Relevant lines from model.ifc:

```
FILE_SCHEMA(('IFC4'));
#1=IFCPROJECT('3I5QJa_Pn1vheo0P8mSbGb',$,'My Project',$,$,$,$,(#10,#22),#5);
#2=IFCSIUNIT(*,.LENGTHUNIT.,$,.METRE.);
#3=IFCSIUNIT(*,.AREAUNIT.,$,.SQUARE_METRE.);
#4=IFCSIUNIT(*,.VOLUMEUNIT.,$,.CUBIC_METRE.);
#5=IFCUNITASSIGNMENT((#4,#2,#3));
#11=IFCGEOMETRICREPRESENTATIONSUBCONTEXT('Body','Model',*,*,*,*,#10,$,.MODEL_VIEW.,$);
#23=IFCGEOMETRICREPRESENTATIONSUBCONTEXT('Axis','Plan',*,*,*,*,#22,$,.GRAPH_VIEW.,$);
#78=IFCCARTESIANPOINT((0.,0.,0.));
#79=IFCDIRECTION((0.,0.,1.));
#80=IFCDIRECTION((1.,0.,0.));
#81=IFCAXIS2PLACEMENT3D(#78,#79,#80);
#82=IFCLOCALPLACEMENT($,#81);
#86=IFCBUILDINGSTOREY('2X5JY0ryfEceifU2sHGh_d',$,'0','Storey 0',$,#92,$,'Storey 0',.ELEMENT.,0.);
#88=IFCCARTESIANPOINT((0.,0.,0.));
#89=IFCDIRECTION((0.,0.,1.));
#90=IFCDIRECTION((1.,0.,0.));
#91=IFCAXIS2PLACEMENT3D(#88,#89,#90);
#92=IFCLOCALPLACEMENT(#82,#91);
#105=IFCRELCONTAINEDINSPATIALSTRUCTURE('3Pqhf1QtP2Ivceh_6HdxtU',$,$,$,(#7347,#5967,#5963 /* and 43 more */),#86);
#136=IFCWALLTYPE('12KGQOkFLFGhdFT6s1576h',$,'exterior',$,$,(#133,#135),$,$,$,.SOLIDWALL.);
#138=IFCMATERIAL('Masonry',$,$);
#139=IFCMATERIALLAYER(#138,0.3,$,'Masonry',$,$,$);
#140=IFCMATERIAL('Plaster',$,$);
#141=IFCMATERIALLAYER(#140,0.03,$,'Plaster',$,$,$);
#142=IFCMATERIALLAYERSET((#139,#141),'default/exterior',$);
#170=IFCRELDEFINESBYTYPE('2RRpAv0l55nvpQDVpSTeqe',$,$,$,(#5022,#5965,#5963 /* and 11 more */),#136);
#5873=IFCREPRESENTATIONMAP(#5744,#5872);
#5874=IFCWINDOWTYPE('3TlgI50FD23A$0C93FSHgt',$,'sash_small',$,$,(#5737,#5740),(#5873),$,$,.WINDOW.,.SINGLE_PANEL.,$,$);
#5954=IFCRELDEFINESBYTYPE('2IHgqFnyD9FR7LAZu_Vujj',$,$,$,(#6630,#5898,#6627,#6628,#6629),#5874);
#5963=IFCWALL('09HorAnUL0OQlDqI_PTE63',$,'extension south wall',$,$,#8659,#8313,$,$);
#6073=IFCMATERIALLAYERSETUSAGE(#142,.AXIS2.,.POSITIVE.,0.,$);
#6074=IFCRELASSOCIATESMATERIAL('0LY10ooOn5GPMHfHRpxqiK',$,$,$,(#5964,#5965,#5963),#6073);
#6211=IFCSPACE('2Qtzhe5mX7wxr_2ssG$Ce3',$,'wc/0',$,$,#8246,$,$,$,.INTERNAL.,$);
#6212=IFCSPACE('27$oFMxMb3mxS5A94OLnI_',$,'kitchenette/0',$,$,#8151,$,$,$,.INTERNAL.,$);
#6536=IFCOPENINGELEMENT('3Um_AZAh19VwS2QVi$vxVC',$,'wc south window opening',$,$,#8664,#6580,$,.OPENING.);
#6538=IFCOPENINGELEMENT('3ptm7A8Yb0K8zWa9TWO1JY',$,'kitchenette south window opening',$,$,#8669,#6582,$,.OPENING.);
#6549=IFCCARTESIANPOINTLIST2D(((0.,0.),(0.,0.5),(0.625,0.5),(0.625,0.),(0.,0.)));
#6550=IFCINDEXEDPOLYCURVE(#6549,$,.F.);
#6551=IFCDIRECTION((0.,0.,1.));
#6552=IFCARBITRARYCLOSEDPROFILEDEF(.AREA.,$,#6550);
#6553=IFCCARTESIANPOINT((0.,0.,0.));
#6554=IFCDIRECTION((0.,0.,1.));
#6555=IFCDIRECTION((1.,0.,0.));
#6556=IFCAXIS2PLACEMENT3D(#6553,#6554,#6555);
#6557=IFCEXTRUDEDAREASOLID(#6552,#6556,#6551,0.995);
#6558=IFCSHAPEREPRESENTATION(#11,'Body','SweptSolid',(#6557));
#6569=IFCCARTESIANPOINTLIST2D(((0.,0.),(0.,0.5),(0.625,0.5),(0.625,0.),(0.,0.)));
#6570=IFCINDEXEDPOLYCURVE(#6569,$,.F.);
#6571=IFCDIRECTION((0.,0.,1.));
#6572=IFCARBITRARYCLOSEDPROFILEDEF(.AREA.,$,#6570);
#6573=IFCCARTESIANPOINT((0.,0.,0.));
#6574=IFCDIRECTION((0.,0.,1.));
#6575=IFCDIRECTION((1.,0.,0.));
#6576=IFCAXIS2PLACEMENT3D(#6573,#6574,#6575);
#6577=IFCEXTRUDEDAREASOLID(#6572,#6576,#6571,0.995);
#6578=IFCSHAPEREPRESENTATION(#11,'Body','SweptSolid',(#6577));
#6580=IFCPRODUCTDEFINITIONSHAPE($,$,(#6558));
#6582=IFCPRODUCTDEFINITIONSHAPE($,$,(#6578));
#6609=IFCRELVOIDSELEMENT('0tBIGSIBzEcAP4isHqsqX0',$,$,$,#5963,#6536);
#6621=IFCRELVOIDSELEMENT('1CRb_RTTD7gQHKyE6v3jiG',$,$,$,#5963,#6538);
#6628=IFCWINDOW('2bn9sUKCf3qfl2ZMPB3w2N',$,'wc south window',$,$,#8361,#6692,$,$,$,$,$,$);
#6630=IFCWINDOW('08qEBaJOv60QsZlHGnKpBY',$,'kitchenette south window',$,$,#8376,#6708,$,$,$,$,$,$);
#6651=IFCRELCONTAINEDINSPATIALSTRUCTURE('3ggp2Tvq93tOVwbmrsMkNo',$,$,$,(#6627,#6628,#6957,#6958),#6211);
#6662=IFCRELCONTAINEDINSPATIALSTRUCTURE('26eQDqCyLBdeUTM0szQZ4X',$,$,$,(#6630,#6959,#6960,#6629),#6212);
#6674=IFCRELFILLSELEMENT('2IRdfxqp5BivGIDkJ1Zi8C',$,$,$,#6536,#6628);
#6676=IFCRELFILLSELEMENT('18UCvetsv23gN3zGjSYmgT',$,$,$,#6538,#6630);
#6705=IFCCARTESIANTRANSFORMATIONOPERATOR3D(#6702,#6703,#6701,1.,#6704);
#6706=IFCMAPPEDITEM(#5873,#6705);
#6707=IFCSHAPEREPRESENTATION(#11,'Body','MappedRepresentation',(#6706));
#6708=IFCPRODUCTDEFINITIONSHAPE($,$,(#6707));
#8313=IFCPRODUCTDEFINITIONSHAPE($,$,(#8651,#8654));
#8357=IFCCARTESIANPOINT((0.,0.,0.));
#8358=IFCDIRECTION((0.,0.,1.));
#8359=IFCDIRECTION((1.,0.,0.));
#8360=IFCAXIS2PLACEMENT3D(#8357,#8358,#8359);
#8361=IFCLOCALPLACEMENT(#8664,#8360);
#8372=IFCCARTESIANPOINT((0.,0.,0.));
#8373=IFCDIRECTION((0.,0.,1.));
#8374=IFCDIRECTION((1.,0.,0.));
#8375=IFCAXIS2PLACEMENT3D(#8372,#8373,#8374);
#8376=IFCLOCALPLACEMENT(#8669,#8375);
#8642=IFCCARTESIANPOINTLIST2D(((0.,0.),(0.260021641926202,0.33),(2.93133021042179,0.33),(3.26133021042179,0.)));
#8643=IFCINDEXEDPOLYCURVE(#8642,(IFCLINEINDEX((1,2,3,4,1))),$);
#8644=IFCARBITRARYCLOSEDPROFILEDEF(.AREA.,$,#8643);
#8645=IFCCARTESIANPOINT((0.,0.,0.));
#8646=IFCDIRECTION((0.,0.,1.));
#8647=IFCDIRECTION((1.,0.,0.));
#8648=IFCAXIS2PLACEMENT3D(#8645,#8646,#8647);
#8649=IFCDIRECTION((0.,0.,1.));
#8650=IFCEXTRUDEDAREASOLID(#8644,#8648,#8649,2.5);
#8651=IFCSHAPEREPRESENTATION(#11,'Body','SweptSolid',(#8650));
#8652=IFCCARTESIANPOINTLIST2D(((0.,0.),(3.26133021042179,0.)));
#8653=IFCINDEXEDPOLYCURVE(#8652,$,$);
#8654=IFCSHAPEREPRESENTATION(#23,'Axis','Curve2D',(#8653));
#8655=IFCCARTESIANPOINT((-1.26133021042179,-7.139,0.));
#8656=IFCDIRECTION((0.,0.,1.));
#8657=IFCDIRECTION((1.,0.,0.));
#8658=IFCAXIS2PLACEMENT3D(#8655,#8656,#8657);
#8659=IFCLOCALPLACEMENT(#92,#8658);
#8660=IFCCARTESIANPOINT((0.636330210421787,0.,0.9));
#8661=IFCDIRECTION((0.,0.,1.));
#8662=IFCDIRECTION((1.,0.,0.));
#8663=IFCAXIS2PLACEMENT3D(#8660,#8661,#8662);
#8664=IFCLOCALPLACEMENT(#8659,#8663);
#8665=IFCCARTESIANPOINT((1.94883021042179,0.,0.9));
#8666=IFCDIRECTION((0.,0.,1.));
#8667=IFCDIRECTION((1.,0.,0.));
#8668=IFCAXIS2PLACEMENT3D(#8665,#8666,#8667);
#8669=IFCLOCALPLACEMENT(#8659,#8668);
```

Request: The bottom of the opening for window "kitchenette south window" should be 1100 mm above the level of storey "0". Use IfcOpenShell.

```python
import numpy as np
import ifcopenshell
import ifcopenshell.api.geometry
import ifcopenshell.geom
import ifcopenshell.util.element
import ifcopenshell.util.placement
import ifcopenshell.util.shape
import ifcopenshell.util.unit

model = ifcopenshell.open("model.ifc")
unit_scale = ifcopenshell.util.unit.calculate_unit_scale(model)

window = model.by_guid("08qEBaJOv60QsZlHGnKpBY")
opening = window.FillsVoids[0].RelatingOpeningElement
storey = ifcopenshell.util.element.get_container(window, ifc_class="IfcBuildingStorey")
level = ifcopenshell.util.placement.get_local_placement(storey.ObjectPlacement)[2, 3]

# The opening's origin need not be at the sill, so measure its lowest point.
shape = ifcopenshell.geom.create_shape(ifcopenshell.geom.settings(), opening)
bottom = ifcopenshell.util.shape.get_shape_bottom_elevation(shape, shape.geometry) / unit_scale
dz = level + 1.1 / unit_scale - bottom

shift = np.array([0.0, 0.0, dz])
# The window is placed relative to its opening, so it follows when the opening moves.
matrix = ifcopenshell.util.placement.get_local_placement(opening.ObjectPlacement)
matrix[:3, 3] += shift
ifcopenshell.api.geometry.edit_object_placement(
    model, product=opening, matrix=matrix, is_si=False, should_transform_children=True
)

print(f"moved by {dz * unit_scale:+.3f} m")

model.write("model_rev.ifc")
```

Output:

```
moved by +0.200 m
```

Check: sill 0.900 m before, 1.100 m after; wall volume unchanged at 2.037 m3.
